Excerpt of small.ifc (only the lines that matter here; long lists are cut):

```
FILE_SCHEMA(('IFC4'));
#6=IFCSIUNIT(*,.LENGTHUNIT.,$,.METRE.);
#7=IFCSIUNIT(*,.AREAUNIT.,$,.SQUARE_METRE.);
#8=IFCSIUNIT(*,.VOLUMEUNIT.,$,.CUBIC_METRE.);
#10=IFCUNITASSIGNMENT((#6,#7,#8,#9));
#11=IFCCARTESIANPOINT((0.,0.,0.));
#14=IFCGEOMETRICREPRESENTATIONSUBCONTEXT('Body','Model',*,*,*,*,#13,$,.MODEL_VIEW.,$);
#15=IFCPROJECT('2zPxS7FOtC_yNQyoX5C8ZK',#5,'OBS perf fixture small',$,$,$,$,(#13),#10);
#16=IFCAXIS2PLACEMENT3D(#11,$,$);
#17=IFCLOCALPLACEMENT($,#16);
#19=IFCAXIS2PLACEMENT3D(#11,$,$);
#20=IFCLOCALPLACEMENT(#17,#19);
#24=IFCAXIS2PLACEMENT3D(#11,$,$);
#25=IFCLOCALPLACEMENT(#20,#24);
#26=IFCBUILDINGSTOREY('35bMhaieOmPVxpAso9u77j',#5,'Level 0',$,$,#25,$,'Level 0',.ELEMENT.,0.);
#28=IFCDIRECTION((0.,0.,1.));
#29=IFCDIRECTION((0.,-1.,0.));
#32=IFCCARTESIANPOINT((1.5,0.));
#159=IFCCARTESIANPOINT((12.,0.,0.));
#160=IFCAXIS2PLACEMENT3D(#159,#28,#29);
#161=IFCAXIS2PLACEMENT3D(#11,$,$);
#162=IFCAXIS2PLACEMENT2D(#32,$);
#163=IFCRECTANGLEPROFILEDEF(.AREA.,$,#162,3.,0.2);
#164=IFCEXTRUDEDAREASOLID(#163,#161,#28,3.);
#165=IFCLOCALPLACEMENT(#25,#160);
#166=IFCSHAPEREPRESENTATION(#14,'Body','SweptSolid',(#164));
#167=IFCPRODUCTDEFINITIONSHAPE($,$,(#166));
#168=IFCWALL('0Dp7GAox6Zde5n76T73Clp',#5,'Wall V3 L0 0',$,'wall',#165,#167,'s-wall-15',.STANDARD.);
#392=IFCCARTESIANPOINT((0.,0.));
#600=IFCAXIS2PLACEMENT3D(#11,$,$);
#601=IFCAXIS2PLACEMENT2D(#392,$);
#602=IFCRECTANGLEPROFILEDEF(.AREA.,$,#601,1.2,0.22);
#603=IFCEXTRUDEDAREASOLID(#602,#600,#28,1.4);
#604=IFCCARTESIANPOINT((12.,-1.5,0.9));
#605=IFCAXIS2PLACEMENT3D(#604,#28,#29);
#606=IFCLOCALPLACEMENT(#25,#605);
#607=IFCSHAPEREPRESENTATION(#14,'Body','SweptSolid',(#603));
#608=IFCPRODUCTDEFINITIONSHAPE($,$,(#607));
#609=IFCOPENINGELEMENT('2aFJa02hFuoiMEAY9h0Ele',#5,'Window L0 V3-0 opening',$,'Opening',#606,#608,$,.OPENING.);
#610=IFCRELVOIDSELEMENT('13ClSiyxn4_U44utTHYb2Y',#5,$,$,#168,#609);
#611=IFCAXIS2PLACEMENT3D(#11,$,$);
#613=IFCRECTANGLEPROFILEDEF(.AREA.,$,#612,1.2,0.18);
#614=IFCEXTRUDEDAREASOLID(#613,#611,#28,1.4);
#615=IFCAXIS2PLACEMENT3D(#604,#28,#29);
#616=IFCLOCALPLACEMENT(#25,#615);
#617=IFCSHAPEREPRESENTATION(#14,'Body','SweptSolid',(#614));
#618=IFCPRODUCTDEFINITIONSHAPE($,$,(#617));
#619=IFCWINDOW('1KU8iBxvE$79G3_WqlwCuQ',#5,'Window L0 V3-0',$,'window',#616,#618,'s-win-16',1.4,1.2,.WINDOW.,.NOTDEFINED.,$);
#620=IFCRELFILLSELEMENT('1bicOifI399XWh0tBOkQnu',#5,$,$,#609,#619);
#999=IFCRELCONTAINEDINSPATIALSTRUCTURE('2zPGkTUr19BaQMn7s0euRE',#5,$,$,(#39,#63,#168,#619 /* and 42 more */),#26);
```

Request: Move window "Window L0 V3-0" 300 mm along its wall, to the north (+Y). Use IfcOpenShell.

```python
import ifcopenshell
import ifcopenshell.api.geometry
import ifcopenshell.util.placement
import ifcopenshell.util.unit

model = ifcopenshell.open("small.ifc")
unit_scale = ifcopenshell.util.unit.calculate_unit_scale(model)

window = model.by_guid("1KU8iBxvE$79G3_WqlwCuQ")
opening = window.FillsVoids[0].RelatingOpeningElement
wall = opening.VoidsElements[0].RelatingBuildingElement

wall_matrix = ifcopenshell.util.placement.get_local_placement(wall.ObjectPlacement)
shift = wall_matrix[:3, 0] * -0.3 / unit_scale
before = ifcopenshell.util.placement.get_local_placement(window.ObjectPlacement)[:3, 3].copy()

# The window is not placed relative to its opening, so move both.
for product in (opening, window):
    matrix = ifcopenshell.util.placement.get_local_placement(product.ObjectPlacement)
    matrix[:3, 3] += shift
    ifcopenshell.api.geometry.edit_object_placement(model, product=product, matrix=matrix, is_si=False)

after = ifcopenshell.util.placement.get_local_placement(window.ObjectPlacement)[:3, 3]
print("window moved by", (after - before).round(3) + 0.0)

model.write("small-out.ifc")
```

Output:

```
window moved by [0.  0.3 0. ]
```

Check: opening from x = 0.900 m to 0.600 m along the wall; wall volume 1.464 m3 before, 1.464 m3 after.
